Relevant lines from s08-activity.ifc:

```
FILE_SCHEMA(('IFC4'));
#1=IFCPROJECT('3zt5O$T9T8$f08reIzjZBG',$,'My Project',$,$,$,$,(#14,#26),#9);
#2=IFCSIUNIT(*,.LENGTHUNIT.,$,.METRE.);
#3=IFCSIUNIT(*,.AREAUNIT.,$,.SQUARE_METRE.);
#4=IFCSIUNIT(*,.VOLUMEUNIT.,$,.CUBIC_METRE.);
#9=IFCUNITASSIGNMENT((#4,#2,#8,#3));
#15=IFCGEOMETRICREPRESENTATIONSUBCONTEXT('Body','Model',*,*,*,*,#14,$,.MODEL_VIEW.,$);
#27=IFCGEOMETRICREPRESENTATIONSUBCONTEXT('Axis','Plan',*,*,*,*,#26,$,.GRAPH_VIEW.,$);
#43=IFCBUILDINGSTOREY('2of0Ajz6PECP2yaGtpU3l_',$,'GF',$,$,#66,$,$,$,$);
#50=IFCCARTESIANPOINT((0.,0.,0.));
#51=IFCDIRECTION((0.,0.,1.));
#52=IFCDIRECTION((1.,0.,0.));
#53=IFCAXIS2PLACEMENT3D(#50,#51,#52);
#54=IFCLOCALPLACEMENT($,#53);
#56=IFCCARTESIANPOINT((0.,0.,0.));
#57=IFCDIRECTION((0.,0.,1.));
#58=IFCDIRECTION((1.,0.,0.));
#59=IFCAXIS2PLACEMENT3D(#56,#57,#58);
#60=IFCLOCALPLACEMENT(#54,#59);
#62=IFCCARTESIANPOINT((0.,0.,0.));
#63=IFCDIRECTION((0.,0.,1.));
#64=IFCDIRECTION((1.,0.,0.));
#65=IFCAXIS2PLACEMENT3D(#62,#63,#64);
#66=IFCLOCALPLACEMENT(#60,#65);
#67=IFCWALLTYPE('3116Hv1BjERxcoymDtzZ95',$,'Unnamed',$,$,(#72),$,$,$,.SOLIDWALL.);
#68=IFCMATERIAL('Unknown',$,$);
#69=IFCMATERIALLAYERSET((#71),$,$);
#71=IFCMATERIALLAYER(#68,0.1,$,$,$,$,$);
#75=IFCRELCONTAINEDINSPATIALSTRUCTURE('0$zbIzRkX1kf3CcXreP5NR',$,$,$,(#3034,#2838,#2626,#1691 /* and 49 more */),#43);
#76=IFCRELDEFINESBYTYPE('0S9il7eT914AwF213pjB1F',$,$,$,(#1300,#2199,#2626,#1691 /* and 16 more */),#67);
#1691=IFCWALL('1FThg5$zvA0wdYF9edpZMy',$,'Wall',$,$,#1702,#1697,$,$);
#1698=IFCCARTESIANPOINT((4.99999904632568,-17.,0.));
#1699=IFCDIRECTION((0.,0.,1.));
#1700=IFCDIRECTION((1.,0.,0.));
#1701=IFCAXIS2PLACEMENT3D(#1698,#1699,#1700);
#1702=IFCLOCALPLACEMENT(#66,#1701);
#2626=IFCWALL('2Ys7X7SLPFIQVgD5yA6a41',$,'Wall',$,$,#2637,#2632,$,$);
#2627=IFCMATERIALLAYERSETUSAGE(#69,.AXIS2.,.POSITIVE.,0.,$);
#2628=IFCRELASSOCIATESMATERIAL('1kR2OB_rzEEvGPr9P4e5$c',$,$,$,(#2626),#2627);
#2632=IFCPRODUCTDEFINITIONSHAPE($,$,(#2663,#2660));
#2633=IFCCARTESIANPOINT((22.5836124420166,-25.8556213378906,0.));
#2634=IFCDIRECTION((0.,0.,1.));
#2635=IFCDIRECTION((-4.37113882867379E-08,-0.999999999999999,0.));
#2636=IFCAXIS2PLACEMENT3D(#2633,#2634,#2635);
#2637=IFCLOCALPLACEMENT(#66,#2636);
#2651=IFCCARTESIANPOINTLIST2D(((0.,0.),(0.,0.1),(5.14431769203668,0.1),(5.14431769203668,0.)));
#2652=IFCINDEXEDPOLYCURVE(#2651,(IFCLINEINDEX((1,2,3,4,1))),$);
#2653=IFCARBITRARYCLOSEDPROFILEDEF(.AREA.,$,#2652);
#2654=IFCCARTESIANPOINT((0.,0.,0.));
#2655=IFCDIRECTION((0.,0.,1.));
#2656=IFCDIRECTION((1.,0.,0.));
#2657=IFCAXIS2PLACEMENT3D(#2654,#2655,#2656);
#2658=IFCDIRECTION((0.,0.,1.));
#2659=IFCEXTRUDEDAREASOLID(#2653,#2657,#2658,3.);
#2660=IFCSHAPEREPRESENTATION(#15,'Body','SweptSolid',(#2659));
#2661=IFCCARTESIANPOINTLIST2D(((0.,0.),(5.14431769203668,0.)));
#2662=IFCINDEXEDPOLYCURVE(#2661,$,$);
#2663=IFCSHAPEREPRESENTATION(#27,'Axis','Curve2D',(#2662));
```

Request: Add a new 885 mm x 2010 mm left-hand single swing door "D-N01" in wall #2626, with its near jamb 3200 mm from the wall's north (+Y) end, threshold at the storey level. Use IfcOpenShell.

```python
import numpy as np
import ifcopenshell
import ifcopenshell.api.feature
import ifcopenshell.api.geometry
import ifcopenshell.api.root
import ifcopenshell.api.spatial
import ifcopenshell.geom
import ifcopenshell.util.element
import ifcopenshell.util.placement
import ifcopenshell.util.representation
import ifcopenshell.util.shape
import ifcopenshell.util.unit

model = ifcopenshell.open("s08-activity.ifc")
unit_scale = ifcopenshell.util.unit.calculate_unit_scale(model)
settings = ifcopenshell.geom.settings()


def volume(element):
    """Net volume in cubic metres, openings subtracted."""
    shape = ifcopenshell.geom.create_shape(settings, element)
    return ifcopenshell.util.shape.get_volume(shape.geometry)


wall = model.by_id(2626)
storey = ifcopenshell.util.element.get_container(wall, ifc_class="IfcBuildingStorey")
context = ifcopenshell.util.representation.get_context(model, "Model", "Body", "MODEL_VIEW")
before = volume(wall)

width, height, from_end, sill = 0.885, 2.01, 3.2, 0.0  # metres

# The wall runs along its own X axis, and the end named is its -X end.
wall_shape = ifcopenshell.geom.create_shape(settings, wall)
x, y, z = ifcopenshell.util.shape.get_vertices(wall_shape.geometry).T
start = x.min() + from_end
face, thickness = float(y.min()), float(y.max() - y.min())
wall_matrix = ifcopenshell.util.placement.get_local_placement(wall.ObjectPlacement)
level = ifcopenshell.util.placement.get_local_placement(storey.ObjectPlacement)[2, 3]


def in_wall(x, y):
    """Placement at x, y metres in the wall's axes, at sill height."""
    matrix = wall_matrix.copy()
    matrix[:, 3] = wall_matrix @ np.array([x / unit_scale, y / unit_scale, 0.0, 1.0])
    matrix[2, 3] = level + sill / unit_scale
    return matrix


# Opening: a box that overshoots both wall faces by 50 mm.
opening = ifcopenshell.api.root.create_entity(model, ifc_class="IfcOpeningElement", predefined_type="OPENING")
box = ifcopenshell.api.geometry.add_wall_representation(
    model, context=context, length=width, height=height, thickness=thickness + 0.1
)
ifcopenshell.api.geometry.assign_representation(model, product=opening, representation=box)
ifcopenshell.api.geometry.edit_object_placement(model, product=opening, matrix=in_wall(start, face - 0.05), is_si=False)
ifcopenshell.api.feature.add_feature(model, feature=opening, element=wall)

door = ifcopenshell.api.root.create_entity(model, ifc_class="IfcDoor", name="D-N01", predefined_type="DOOR")
door.OverallWidth, door.OverallHeight = width / unit_scale, height / unit_scale
door.OperationType = "SINGLE_SWING_LEFT"
body = ifcopenshell.api.geometry.add_door_representation(
    model,
    context=context,
    overall_width=door.OverallWidth,
    overall_height=door.OverallHeight,
    operation_type="SINGLE_SWING_LEFT",
    lining_properties={"LiningDepth": thickness / unit_scale, "ThresholdDepth": thickness / unit_scale},
)
ifcopenshell.api.geometry.assign_representation(model, product=door, representation=body)
ifcopenshell.api.spatial.assign_container(model, products=[door], relating_structure=storey)
ifcopenshell.api.feature.add_filling(model, opening=opening, element=door)

# The lining spans the wall, so the door starts at the wall face.
ifcopenshell.api.geometry.edit_object_placement(model, product=door, matrix=in_wall(start, face), is_si=False)

after = volume(wall)

print(f"wall volume {before:.3f} -> {after:.3f} m3")

model.write("s08-activity_v2.ifc")
```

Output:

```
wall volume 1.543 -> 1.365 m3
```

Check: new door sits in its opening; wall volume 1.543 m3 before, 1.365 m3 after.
